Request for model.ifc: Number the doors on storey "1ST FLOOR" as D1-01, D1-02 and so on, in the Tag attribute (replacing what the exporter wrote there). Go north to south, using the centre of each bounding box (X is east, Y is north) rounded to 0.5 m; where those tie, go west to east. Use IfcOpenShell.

First a look at what the model holds.

```python
import ifcopenshell
import ifcopenshell.util.element
import ifcopenshell.util.placement

model = ifcopenshell.open("model.ifc")
print(model.schema)
storey = next(s for s in model.by_type("IfcBuildingStorey") if s.Name == "1ST FLOOR")
doors = [e for e in ifcopenshell.util.element.get_decomposition(storey) if e.is_a("IfcDoor")]
for e in sorted(doors, key=lambda e: e.id()):
    origin = ifcopenshell.util.placement.get_local_placement(e.ObjectPlacement)[:3, 3]
    print(e.id(), e.Tag, e.Name, origin.round(2) + 0.0, sep=" | ")
```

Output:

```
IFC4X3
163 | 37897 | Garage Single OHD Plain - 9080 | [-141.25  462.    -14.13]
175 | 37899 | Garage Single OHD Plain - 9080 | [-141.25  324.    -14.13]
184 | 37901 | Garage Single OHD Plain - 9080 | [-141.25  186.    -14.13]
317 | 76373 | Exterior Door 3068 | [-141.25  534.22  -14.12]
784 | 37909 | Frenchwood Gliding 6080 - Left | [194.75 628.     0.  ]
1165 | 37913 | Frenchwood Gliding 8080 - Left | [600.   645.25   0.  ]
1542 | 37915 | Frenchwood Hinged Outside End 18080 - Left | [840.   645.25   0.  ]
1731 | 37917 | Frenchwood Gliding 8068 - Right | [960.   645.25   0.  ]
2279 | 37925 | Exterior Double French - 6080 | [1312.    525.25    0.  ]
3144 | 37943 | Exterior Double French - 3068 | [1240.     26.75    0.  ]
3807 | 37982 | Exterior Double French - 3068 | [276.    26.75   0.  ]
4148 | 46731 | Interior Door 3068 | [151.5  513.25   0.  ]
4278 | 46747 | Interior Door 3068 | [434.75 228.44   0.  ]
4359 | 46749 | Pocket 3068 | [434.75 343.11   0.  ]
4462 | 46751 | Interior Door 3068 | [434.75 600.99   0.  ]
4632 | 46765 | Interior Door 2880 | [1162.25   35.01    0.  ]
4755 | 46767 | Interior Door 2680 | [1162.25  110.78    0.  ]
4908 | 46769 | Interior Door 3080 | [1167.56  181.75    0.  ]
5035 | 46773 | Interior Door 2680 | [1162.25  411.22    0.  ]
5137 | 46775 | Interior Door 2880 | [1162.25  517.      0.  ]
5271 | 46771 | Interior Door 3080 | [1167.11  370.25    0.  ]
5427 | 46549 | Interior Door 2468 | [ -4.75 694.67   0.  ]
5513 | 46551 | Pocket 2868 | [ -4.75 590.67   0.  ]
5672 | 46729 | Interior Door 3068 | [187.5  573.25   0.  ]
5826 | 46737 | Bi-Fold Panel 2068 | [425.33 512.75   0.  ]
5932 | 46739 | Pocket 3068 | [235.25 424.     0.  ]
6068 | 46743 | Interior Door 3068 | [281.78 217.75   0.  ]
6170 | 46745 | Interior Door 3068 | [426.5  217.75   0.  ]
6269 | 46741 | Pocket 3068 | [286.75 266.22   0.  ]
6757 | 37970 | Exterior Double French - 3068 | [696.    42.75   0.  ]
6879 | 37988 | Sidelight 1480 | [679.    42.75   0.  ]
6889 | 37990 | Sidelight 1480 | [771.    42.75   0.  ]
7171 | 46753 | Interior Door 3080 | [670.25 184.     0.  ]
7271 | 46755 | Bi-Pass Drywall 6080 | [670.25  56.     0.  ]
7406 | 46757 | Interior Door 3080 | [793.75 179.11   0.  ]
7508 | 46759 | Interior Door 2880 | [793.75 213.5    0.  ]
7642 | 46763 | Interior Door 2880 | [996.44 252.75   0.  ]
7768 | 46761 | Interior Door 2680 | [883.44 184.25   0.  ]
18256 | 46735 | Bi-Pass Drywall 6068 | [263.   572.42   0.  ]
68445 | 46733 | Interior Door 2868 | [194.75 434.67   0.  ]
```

```python
import ifcopenshell
import ifcopenshell.geom
import ifcopenshell.util.element
import ifcopenshell.util.shape

model = ifcopenshell.open("model.ifc")
settings = ifcopenshell.geom.settings()
settings.set("use-world-coords", True)


def centre(element):
    shape = ifcopenshell.geom.create_shape(settings, element)
    return ifcopenshell.util.shape.get_bbox_centroid(shape.geometry)


storey = next(s for s in model.by_type("IfcBuildingStorey") if s.Name == "1ST FLOOR")
doors = [e for e in ifcopenshell.util.element.get_decomposition(storey) if e.is_a("IfcDoor")]

# Insertion points can sit at a corner or the storey origin, so sort by the geometry (in metres).
centres = {e: centre(e) for e in doors}
doors.sort(key=lambda e: (-round(centres[e][1] / 0.5), centres[e][0]))

for i, e in enumerate(doors, start=1):
    number = f"D1-{i:02d}"
    e.Tag = number
    print(e.id(), number)

model.write("model_updated.ifc")
```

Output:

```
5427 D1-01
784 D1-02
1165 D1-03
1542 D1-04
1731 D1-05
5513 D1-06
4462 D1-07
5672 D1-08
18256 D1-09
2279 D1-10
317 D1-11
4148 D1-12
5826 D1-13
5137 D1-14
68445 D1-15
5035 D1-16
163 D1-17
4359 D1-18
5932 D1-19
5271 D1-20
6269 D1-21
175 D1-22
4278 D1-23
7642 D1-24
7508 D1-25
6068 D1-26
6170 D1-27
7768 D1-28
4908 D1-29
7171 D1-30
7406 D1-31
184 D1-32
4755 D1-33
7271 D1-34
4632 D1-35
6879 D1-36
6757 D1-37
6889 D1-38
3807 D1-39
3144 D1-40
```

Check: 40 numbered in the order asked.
